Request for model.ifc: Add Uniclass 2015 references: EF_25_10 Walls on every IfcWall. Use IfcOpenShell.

First a look at what the model holds.

```python
import ifcopenshell

model = ifcopenshell.open("model.ifc")
print(model.schema)
print("classifications:", [c.Name for c in model.by_type("IfcClassification")])
for ifc_class in ("IfcDoor", "IfcRoof", "IfcStair", "IfcWall", "IfcWindow"):
    print(ifc_class, len(model.by_type(ifc_class)))
```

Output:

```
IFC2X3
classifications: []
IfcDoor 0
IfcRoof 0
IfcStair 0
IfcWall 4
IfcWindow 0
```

```python
import ifcopenshell
import ifcopenshell.api.classification

model = ifcopenshell.open("model.ifc")

# IFC2X3 requires Source and Edition and has no link from the project to the system.
system = model.create_entity("IfcClassification", Source="NBS", Edition="2015", Name="Uniclass 2015")

codes = {
    "IfcWall": ("EF_25_10", "Walls"),
}
for ifc_class, (code, name) in codes.items():
    products = model.by_type(ifc_class)
    ifcopenshell.api.classification.add_reference(
        model, products=products, classification=system, identification=code, name=name
    )
    print(code, len(products))

model.write("model_edited.ifc")
```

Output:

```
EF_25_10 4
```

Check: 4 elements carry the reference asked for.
